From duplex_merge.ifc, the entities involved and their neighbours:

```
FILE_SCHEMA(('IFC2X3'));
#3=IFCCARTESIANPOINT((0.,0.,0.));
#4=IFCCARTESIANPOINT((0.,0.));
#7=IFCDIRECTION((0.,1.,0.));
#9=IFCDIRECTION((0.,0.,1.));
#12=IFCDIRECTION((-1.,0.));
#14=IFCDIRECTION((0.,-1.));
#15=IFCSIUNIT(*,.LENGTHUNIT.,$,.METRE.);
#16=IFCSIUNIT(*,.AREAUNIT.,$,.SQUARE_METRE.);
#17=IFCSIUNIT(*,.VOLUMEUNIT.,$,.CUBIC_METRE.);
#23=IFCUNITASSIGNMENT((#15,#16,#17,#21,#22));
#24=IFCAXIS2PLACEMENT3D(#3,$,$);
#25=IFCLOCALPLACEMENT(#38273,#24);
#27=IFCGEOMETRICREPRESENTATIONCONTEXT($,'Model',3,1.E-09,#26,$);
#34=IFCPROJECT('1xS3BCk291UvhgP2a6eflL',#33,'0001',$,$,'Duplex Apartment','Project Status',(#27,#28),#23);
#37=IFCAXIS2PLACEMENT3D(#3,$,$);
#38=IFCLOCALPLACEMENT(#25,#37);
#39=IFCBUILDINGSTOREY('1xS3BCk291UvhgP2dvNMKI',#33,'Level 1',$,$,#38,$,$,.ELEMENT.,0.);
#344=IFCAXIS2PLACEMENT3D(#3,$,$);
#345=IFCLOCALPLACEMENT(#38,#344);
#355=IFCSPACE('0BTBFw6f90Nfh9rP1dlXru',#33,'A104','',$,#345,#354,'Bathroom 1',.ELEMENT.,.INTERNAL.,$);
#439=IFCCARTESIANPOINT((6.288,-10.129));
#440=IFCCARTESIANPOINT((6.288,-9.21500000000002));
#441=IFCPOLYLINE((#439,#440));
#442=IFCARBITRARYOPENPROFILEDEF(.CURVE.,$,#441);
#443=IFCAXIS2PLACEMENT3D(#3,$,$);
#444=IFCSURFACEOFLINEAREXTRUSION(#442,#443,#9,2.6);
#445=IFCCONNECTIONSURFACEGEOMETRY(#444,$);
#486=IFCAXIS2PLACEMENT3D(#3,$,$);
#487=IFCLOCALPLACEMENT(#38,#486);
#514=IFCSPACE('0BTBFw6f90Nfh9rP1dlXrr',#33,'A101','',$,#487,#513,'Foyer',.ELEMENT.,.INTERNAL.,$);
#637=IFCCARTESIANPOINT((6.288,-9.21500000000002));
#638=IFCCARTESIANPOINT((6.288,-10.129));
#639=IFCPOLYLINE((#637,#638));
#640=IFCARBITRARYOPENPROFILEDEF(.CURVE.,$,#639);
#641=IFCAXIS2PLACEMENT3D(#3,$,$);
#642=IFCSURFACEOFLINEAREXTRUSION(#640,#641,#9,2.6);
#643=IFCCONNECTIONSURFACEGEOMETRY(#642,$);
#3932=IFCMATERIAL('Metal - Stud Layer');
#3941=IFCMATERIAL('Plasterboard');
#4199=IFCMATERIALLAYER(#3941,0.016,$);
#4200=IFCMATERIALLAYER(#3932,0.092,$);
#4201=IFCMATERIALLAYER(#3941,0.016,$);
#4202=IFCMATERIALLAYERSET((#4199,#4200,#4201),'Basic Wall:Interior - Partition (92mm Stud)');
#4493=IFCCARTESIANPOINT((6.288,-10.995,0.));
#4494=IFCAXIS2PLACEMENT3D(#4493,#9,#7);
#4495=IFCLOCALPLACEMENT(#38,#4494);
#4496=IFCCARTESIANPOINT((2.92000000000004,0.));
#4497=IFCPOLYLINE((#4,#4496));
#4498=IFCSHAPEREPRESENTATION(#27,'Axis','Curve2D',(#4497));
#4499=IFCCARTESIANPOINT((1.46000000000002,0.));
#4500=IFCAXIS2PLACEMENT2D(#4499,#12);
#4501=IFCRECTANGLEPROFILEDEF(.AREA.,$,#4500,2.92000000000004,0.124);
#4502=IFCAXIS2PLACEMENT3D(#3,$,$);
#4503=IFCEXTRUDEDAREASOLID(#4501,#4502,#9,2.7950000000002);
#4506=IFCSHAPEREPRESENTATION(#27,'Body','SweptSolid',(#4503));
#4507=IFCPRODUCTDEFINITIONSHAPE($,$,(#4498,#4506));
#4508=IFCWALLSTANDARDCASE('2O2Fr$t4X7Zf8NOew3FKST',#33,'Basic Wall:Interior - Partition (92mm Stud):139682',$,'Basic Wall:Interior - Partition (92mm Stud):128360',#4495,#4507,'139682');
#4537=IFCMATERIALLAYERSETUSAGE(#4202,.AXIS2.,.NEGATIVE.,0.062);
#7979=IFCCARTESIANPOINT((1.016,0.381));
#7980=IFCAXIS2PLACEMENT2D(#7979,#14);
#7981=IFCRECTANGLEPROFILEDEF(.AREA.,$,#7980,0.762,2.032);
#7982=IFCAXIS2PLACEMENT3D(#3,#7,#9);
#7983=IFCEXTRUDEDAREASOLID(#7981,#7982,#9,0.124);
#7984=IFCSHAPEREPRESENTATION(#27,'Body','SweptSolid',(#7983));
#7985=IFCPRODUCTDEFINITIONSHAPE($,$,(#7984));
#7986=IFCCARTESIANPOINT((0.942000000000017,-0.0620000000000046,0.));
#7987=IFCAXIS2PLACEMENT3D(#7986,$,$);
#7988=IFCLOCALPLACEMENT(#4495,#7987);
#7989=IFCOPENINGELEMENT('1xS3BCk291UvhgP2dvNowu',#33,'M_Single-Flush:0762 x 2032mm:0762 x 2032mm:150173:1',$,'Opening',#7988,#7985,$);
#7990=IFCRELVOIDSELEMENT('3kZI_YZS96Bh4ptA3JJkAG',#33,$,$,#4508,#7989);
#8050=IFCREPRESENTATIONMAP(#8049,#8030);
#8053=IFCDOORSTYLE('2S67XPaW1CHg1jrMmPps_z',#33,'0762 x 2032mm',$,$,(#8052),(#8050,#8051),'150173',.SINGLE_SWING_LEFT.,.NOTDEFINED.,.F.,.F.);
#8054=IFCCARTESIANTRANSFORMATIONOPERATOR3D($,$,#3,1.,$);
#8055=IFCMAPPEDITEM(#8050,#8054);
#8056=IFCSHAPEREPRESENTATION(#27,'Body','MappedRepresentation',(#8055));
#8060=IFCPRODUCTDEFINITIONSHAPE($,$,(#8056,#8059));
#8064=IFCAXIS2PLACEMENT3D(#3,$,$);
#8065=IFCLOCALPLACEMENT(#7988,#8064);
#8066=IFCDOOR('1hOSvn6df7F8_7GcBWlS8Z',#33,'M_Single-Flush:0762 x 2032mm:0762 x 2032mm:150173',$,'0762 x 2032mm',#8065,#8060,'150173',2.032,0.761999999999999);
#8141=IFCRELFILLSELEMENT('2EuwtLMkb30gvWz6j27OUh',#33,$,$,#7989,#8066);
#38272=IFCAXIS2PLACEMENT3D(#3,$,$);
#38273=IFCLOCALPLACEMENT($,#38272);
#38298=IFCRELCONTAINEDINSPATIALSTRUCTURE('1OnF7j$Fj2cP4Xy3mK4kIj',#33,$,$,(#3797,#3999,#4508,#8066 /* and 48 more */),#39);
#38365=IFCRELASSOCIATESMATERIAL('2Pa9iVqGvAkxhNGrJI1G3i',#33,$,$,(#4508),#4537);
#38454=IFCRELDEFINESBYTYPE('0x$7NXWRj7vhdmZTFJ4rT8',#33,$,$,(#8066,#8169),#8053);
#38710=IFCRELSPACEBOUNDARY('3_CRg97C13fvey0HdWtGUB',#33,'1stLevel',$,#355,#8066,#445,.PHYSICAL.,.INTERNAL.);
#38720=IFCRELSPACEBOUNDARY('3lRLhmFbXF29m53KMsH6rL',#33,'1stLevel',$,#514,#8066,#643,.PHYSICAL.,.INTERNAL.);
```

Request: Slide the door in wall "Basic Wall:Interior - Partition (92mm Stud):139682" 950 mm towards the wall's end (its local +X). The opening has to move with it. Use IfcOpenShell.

```python
import numpy as np
import ifcopenshell
import ifcopenshell.api.geometry
import ifcopenshell.util.placement
import ifcopenshell.util.unit

model = ifcopenshell.open("duplex_merge.ifc")
unit_scale = ifcopenshell.util.unit.calculate_unit_scale(model)

door = model.by_guid("1hOSvn6df7F8_7GcBWlS8Z")
opening = door.FillsVoids[0].RelatingOpeningElement
wall = opening.VoidsElements[0].RelatingBuildingElement

wall_matrix = ifcopenshell.util.placement.get_local_placement(wall.ObjectPlacement)
shift = wall_matrix[:3, 0] * 0.95 / unit_scale
before = ifcopenshell.util.placement.get_local_placement(door.ObjectPlacement)[:3, 3].copy()

# The door is placed relative to its opening, so it follows when the opening moves.
matrix = ifcopenshell.util.placement.get_local_placement(opening.ObjectPlacement)
matrix[:3, 3] += shift
ifcopenshell.api.geometry.edit_object_placement(
    model, product=opening, matrix=matrix, is_si=False, should_transform_children=True
)

# Space boundary surfaces are stored in each space's coordinates; move them too.
for rel in door.ProvidesBoundaries:
    if not rel.ConnectionGeometry:
        continue
    surface = rel.ConnectionGeometry.SurfaceOnRelatingElement
    space_matrix = ifcopenshell.util.placement.get_local_placement(rel.RelatingSpace.ObjectPlacement)
    point = np.array(surface.Position.Location.Coordinates) + space_matrix[:3, :3].T @ shift
    surface.Position = model.createIfcAxis2Placement3D(
        model.createIfcCartesianPoint(point.tolist()), surface.Position.Axis, surface.Position.RefDirection
    )

after = ifcopenshell.util.placement.get_local_placement(door.ObjectPlacement)[:3, 3]
print("door moved by", (after - before).round(3) + 0.0)

model.write("duplex_merge_v2.ifc")
```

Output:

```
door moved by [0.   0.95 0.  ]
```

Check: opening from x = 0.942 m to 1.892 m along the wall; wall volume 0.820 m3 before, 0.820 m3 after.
